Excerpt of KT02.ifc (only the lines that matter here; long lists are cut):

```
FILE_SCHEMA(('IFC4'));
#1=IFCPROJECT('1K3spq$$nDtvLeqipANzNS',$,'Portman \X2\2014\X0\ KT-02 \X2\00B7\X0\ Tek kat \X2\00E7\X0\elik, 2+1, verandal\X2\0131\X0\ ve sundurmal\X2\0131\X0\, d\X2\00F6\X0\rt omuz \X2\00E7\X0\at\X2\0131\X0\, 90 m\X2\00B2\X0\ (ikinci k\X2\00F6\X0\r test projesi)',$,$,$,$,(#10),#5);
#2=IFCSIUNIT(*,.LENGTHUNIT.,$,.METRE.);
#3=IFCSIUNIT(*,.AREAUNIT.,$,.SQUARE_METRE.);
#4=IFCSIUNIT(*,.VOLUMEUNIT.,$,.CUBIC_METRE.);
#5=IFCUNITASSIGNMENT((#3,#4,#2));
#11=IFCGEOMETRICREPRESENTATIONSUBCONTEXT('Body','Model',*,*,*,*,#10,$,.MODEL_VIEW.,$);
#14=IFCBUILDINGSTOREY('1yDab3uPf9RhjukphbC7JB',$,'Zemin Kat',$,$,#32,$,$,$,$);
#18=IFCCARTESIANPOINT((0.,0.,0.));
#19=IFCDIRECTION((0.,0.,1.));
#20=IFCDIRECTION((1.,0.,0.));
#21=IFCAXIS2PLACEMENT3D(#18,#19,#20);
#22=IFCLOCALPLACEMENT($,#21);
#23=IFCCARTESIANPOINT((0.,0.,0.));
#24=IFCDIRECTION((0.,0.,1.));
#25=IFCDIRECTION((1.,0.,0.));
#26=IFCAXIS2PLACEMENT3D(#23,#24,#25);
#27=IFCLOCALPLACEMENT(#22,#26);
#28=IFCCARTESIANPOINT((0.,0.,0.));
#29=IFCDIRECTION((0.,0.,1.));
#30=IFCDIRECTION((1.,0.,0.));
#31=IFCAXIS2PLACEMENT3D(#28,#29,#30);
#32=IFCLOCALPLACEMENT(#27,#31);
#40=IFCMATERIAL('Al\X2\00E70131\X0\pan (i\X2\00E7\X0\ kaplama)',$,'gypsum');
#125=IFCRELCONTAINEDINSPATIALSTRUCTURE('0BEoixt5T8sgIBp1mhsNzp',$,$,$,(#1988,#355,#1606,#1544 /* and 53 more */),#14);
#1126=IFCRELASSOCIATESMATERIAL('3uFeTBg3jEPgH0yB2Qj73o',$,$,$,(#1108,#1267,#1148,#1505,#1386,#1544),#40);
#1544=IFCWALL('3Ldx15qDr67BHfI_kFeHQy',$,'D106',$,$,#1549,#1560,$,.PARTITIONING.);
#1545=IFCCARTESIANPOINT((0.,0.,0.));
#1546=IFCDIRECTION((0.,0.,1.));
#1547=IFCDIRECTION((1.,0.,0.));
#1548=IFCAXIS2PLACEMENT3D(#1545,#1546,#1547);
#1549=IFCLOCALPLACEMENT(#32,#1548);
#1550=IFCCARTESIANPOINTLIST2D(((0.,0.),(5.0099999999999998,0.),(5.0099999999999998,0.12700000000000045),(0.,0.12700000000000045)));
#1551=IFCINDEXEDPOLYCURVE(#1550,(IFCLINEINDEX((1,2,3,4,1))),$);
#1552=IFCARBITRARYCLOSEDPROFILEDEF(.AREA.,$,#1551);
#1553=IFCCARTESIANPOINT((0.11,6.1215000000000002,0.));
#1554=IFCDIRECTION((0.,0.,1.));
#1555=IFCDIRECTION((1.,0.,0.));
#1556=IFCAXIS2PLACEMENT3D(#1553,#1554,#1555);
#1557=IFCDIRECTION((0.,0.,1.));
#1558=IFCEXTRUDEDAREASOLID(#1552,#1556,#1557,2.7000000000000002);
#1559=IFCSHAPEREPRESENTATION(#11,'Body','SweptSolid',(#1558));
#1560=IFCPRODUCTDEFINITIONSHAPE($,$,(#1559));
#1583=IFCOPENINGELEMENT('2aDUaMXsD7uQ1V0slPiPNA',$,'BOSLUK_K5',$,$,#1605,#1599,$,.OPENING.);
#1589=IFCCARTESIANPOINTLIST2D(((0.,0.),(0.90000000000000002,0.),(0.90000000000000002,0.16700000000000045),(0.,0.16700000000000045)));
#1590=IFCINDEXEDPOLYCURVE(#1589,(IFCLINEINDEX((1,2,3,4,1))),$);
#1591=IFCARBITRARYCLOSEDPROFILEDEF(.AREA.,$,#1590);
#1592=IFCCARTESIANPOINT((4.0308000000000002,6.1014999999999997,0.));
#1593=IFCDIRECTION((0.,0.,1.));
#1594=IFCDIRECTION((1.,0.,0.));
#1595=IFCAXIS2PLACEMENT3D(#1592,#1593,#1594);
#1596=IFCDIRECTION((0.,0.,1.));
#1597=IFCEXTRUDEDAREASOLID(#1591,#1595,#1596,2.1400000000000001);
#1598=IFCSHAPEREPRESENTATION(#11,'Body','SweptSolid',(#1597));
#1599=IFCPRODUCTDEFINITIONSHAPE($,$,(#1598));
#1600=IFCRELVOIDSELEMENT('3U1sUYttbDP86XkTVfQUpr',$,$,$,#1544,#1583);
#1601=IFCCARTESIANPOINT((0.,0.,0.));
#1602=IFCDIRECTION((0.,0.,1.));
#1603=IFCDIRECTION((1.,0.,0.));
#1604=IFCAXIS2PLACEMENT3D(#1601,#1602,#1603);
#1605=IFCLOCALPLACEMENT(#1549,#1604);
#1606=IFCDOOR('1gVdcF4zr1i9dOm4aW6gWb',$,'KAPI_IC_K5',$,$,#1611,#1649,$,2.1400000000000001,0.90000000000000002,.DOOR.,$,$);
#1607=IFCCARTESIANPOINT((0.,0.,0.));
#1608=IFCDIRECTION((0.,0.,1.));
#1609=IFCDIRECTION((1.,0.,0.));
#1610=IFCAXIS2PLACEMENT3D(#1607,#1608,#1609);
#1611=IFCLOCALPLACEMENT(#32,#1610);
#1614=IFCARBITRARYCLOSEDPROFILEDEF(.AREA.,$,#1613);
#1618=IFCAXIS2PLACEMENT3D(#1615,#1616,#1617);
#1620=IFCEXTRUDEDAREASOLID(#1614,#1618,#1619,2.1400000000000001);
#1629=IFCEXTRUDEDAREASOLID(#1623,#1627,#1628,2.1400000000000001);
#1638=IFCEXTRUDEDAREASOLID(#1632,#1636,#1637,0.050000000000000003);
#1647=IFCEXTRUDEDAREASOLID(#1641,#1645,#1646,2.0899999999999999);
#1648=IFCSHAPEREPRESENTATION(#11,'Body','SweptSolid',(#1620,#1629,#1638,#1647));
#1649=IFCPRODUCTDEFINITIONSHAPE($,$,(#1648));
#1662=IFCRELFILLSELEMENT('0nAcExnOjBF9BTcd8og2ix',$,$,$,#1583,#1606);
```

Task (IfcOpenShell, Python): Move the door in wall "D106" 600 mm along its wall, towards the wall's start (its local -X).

```python
import ifcopenshell
import ifcopenshell.api.geometry
import ifcopenshell.util.placement
import ifcopenshell.util.unit

model = ifcopenshell.open("KT02.ifc")
unit_scale = ifcopenshell.util.unit.calculate_unit_scale(model)

door = model.by_id(1606)
opening = door.FillsVoids[0].RelatingOpeningElement
wall = opening.VoidsElements[0].RelatingBuildingElement

wall_matrix = ifcopenshell.util.placement.get_local_placement(wall.ObjectPlacement)
shift = wall_matrix[:3, 0] * -0.6 / unit_scale
before = ifcopenshell.util.placement.get_local_placement(door.ObjectPlacement)[:3, 3].copy()

# The door is not placed relative to its opening, so move both.
for product in (opening, door):
    matrix = ifcopenshell.util.placement.get_local_placement(product.ObjectPlacement)
    matrix[:3, 3] += shift
    ifcopenshell.api.geometry.edit_object_placement(model, product=product, matrix=matrix, is_si=False)

after = ifcopenshell.util.placement.get_local_placement(door.ObjectPlacement)[:3, 3]
print("door moved by", (after - before).round(3) + 0.0)

model.write("KT02_rev.ifc")
```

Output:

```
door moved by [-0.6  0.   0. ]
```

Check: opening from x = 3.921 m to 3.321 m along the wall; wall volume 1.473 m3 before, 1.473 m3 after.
